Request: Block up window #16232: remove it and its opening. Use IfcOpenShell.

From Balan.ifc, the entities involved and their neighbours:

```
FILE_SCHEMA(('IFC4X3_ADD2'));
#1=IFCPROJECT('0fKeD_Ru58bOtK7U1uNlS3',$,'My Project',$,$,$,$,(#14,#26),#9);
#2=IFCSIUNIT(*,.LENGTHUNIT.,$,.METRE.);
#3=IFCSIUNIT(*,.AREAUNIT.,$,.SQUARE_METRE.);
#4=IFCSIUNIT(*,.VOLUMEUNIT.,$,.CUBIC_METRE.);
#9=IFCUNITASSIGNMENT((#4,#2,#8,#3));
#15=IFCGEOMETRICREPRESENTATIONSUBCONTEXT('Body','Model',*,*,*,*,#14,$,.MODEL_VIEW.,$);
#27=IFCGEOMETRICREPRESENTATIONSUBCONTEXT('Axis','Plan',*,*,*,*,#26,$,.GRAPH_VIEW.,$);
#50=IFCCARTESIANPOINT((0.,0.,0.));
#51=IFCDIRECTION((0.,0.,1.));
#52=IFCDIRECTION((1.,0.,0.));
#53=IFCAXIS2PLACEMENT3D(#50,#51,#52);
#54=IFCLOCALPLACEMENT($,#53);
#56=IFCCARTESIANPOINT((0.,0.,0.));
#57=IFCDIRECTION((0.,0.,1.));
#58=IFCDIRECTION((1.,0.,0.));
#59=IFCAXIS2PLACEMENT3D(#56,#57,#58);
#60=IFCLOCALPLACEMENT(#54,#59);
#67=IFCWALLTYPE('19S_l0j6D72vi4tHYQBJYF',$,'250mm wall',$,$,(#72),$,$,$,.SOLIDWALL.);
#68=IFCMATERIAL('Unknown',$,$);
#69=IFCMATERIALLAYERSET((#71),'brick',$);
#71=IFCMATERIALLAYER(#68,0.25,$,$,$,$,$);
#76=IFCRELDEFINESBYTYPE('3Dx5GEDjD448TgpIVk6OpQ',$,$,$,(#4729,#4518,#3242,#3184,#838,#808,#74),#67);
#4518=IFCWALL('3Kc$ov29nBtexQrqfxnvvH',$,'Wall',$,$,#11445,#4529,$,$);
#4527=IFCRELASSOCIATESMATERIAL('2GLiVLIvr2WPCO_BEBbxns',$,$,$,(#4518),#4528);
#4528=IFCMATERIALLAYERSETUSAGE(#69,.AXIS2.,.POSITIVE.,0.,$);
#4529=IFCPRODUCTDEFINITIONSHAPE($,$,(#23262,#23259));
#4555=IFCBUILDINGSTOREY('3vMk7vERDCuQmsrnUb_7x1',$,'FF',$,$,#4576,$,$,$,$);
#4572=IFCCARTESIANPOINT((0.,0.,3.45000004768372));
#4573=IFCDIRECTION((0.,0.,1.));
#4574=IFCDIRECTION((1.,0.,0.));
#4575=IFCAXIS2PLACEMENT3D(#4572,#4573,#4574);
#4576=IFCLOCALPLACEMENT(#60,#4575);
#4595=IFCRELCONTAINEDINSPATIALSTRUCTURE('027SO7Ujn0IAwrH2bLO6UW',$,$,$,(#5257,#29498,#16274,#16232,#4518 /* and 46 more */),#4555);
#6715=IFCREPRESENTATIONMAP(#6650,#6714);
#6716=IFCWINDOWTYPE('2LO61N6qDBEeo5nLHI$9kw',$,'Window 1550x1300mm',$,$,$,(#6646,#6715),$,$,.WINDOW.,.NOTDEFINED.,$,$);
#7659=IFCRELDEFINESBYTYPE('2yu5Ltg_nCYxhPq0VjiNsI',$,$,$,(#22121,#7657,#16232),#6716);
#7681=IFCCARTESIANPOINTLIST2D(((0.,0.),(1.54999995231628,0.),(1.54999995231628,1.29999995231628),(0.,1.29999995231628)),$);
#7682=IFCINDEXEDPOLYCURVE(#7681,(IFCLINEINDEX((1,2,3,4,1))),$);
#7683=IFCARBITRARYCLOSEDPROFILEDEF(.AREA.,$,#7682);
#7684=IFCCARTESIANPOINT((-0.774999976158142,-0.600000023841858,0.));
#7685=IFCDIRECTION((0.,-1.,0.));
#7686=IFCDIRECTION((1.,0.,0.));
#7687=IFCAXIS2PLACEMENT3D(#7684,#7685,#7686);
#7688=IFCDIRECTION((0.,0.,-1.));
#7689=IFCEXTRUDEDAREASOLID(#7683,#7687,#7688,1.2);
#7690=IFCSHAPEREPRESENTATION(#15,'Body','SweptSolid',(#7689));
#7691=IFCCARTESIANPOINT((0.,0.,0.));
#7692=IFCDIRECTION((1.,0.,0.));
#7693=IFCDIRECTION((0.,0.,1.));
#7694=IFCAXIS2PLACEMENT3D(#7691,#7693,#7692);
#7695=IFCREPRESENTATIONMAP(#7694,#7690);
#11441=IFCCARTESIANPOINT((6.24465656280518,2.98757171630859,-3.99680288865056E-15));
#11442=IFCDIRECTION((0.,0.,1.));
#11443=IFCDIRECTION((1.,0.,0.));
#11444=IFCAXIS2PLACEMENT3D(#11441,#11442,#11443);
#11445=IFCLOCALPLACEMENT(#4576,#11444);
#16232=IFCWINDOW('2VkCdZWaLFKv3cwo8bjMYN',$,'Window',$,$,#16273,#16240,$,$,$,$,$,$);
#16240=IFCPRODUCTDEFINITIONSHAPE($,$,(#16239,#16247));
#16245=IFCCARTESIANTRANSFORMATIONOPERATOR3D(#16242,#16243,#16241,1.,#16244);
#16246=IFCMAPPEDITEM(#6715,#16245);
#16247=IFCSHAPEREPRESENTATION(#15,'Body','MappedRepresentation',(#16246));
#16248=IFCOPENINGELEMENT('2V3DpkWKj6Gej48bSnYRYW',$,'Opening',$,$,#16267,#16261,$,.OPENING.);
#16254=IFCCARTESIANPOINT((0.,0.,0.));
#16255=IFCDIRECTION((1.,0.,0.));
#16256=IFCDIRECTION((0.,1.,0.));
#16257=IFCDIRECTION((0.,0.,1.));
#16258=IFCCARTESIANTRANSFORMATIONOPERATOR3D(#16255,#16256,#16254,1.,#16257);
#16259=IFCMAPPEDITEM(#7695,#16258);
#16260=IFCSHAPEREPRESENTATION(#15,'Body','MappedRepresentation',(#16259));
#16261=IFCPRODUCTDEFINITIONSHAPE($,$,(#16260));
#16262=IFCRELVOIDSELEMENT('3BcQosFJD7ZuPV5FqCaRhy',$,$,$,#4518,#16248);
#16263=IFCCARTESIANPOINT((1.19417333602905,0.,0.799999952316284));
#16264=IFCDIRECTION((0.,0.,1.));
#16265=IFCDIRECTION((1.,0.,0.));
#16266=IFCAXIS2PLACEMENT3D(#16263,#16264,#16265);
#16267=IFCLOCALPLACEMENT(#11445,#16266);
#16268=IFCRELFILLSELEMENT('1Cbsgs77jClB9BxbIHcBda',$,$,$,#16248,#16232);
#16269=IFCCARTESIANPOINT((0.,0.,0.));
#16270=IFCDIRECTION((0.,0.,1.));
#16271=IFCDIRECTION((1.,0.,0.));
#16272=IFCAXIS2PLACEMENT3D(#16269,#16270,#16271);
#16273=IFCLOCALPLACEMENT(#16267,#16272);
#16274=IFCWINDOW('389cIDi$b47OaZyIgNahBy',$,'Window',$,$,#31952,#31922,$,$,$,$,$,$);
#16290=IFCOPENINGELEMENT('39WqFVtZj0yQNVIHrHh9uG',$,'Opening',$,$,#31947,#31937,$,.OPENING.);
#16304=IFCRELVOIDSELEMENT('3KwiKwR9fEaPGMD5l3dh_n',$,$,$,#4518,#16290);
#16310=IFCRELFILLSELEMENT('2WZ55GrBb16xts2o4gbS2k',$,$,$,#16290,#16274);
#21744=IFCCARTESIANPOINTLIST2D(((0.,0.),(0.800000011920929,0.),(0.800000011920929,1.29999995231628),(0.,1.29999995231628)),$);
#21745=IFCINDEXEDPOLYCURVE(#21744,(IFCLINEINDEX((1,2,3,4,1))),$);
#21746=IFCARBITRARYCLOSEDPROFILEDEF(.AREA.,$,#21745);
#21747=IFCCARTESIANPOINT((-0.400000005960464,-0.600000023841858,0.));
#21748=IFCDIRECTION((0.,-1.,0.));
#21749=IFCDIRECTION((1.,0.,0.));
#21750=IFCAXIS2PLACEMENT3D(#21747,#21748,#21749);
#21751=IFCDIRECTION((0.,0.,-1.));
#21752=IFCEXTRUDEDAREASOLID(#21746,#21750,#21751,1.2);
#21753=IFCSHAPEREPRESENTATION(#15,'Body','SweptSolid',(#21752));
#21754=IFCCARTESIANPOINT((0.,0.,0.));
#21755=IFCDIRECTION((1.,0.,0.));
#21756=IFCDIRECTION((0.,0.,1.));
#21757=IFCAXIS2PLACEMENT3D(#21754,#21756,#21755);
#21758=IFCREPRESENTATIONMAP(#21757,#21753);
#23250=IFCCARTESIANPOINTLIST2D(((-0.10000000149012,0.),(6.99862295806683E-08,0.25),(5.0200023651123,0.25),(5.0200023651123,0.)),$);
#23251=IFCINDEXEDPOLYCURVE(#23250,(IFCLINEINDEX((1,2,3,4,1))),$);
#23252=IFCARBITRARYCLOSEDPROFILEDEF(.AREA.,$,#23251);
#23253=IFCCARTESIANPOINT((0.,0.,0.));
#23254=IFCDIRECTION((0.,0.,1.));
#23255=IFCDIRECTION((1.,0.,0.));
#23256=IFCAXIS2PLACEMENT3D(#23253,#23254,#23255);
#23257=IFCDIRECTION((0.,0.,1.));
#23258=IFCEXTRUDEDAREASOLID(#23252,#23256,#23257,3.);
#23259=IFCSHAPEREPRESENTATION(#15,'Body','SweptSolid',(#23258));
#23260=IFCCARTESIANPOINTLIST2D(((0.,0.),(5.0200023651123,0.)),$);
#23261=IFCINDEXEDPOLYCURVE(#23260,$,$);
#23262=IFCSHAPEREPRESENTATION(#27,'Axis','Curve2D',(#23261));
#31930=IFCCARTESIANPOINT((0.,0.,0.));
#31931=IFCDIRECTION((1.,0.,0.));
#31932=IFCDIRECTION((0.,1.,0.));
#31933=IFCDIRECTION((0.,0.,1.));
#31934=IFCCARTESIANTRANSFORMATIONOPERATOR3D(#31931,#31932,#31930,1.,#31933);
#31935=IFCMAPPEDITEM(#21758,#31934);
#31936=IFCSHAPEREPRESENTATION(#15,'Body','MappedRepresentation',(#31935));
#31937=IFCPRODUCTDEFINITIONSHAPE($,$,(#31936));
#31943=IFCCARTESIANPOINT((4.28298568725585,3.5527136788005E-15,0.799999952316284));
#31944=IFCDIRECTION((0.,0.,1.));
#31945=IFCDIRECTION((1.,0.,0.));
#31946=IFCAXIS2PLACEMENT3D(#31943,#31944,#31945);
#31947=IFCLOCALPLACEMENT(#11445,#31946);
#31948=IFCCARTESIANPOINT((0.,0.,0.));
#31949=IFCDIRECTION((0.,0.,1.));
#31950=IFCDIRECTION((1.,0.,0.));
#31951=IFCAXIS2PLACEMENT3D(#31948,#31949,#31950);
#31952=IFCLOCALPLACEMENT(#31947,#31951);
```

```python
import ifcopenshell
import ifcopenshell.api.feature
import ifcopenshell.api.root
import ifcopenshell.geom
import ifcopenshell.util.shape

model = ifcopenshell.open("Balan.ifc")
settings = ifcopenshell.geom.settings()


def volume(element):
    """Net volume in cubic metres, openings subtracted."""
    shape = ifcopenshell.geom.create_shape(settings, element)
    return ifcopenshell.util.shape.get_volume(shape.geometry)


window = model.by_guid("2VkCdZWaLFKv3cwo8bjMYN")
opening = window.FillsVoids[0].RelatingOpeningElement
wall = opening.VoidsElements[0].RelatingBuildingElement
before = volume(wall)

ifcopenshell.api.root.remove_product(model, product=window)
ifcopenshell.api.feature.remove_feature(model, feature=opening)

after = volume(wall)

print(f"wall volume {before:.3f} -> {after:.3f} m3")

model.write("Balan_rev.ifc")
```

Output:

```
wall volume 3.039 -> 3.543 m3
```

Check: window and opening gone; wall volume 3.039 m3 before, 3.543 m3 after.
